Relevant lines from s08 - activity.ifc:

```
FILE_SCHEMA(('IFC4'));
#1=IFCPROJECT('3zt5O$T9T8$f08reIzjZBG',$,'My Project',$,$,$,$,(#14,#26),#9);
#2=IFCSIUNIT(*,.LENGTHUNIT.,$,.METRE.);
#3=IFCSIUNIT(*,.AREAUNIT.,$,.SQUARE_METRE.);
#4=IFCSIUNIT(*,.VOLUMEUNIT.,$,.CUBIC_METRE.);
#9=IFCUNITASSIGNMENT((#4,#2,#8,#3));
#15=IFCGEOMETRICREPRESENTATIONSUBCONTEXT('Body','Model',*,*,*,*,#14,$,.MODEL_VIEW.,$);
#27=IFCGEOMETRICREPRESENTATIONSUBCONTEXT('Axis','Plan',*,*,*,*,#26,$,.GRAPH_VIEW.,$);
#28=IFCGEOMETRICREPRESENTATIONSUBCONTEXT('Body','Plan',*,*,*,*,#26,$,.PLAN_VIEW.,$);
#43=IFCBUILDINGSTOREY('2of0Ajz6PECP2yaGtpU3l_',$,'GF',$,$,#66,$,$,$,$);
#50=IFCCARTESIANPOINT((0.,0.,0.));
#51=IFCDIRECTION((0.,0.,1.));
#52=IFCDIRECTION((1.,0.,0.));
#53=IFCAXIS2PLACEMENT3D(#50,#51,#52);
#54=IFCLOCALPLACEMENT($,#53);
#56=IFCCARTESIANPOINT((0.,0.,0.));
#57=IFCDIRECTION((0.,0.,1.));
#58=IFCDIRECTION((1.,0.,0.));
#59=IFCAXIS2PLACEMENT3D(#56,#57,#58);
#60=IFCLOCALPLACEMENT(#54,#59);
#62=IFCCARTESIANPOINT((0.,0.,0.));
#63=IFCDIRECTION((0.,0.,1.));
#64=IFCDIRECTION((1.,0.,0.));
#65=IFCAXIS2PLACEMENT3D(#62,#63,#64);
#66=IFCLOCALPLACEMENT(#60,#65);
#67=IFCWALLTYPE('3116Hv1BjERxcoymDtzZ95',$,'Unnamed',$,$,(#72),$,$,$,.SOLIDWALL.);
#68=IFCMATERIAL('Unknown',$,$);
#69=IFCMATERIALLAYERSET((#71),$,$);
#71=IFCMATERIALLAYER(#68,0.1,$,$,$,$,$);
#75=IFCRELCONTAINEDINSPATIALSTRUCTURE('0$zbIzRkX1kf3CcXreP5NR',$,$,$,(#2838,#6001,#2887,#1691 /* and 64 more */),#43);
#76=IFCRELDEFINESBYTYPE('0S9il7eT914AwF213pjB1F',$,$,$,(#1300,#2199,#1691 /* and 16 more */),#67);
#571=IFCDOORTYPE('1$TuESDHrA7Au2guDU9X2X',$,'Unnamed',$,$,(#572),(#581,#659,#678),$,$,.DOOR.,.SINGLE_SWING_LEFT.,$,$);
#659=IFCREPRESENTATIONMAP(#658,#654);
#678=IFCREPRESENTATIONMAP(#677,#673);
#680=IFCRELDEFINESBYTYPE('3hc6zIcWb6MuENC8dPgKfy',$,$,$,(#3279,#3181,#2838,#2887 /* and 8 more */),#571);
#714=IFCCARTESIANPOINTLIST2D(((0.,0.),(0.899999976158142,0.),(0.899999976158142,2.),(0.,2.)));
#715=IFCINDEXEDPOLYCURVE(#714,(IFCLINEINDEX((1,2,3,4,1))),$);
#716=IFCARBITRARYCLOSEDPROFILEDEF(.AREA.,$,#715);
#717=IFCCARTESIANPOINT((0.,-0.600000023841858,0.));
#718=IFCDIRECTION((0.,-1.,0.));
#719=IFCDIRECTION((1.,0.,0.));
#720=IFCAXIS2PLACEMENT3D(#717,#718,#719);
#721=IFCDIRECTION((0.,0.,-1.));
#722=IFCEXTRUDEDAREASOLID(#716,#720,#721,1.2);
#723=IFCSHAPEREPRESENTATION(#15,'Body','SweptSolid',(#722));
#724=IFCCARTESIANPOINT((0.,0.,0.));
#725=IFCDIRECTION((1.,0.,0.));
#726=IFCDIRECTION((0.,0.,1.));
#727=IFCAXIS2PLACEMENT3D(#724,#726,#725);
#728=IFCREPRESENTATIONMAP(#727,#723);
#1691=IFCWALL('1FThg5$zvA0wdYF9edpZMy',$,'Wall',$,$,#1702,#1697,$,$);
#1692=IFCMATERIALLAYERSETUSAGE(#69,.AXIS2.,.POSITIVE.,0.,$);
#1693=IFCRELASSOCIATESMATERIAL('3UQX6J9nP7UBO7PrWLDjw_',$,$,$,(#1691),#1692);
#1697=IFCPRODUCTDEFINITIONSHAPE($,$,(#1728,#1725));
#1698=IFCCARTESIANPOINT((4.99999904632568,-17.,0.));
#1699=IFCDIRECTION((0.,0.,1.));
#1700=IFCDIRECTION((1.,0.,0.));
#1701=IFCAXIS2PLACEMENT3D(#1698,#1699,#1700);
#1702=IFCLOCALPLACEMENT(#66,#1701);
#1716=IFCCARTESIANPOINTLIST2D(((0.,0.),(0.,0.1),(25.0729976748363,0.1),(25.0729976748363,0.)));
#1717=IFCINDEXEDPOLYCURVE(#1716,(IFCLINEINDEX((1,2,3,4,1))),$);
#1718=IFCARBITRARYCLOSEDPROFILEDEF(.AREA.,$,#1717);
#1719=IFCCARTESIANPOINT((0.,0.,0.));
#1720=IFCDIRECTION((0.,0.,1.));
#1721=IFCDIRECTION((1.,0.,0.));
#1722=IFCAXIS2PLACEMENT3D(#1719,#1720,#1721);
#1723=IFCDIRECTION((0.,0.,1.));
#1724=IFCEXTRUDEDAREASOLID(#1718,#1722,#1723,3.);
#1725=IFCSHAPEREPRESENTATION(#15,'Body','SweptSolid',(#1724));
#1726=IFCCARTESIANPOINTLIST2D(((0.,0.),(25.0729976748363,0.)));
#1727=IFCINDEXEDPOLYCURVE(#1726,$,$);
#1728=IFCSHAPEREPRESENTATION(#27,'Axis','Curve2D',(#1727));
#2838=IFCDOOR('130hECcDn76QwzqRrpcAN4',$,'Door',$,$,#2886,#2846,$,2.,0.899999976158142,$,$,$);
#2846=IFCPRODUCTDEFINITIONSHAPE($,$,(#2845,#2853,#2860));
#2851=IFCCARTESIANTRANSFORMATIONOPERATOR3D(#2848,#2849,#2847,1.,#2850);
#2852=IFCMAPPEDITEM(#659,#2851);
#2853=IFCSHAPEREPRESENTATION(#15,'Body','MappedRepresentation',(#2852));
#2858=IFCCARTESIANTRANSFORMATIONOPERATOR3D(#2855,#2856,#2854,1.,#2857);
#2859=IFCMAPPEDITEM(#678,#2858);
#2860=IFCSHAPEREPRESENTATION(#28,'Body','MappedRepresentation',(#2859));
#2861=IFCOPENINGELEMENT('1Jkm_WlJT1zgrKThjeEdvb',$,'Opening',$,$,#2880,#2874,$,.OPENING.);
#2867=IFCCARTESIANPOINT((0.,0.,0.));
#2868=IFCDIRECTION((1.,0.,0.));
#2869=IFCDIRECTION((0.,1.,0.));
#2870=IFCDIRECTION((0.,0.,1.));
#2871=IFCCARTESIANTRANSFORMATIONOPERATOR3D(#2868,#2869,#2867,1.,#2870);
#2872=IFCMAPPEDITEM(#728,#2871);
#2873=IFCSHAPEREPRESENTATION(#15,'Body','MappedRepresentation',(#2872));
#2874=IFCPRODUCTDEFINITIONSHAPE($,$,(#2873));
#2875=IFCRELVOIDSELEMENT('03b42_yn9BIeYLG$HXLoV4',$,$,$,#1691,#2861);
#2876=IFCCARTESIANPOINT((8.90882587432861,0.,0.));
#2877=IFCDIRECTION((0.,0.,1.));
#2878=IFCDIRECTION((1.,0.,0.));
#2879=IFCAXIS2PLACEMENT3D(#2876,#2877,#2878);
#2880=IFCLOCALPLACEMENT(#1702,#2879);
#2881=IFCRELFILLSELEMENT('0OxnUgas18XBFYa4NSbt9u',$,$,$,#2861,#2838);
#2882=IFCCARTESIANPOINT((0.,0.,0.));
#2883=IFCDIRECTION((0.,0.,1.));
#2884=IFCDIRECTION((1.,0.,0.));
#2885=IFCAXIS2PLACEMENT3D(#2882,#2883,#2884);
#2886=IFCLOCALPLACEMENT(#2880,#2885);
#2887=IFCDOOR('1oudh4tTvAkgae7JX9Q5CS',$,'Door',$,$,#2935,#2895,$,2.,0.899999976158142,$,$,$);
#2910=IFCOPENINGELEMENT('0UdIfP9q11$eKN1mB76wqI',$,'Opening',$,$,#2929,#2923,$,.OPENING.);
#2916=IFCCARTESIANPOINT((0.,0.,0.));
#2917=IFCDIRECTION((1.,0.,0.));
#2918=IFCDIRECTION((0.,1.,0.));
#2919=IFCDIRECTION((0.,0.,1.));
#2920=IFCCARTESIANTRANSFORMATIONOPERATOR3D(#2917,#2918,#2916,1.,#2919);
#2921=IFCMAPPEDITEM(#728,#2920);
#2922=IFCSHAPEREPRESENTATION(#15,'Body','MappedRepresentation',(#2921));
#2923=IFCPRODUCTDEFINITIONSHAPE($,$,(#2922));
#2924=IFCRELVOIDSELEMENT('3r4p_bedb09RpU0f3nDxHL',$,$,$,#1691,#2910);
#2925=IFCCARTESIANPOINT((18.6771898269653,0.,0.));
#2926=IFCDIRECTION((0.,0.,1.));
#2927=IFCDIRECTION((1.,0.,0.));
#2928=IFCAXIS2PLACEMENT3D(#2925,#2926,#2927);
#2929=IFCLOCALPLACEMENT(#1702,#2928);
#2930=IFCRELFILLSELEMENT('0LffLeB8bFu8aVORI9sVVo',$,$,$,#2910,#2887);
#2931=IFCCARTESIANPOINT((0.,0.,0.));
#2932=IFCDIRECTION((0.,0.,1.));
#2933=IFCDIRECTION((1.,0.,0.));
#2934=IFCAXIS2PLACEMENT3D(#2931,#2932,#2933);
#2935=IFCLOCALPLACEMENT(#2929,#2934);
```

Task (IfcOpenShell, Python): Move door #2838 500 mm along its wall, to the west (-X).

```python
import ifcopenshell
import ifcopenshell.api.geometry
import ifcopenshell.util.placement

model = ifcopenshell.open("s08 - activity.ifc")

door = model.by_guid("130hECcDn76QwzqRrpcAN4")
opening = door.FillsVoids[0].RelatingOpeningElement
wall = opening.VoidsElements[0].RelatingBuildingElement

wall_matrix = ifcopenshell.util.placement.get_local_placement(wall.ObjectPlacement)
shift = wall_matrix[:3, 0] * -0.5
before = ifcopenshell.util.placement.get_local_placement(door.ObjectPlacement)[:3, 3].copy()

# The door is placed relative to its opening, so it follows when the opening moves.
matrix = ifcopenshell.util.placement.get_local_placement(opening.ObjectPlacement)
matrix[:3, 3] += shift
ifcopenshell.api.geometry.edit_object_placement(
    model, product=opening, matrix=matrix, is_si=False, should_transform_children=True
)

after = ifcopenshell.util.placement.get_local_placement(door.ObjectPlacement)[:3, 3]
print("door moved by", (after - before).round(3) + 0.0)

model.write("s08 - activity-out.ifc")
```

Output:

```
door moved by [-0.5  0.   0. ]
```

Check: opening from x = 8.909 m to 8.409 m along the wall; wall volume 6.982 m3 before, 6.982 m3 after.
